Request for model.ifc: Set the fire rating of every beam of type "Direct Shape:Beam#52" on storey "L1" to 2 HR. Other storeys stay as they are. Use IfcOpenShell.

First a look at what the model holds.

```python
import ifcopenshell
import ifcopenshell.util.element

model = ifcopenshell.open("model.ifc")
print(model.schema)
storey = next(s for s in model.by_type("IfcBuildingStorey") if s.Name == "L1")
beams = [e for e in ifcopenshell.util.element.get_decomposition(storey) if e.is_a("IfcBeam")]
seen = {}
for e in beams:
    element_type = ifcopenshell.util.element.get_type(e)
    key = (element_type.Name if element_type != e and element_type else None, ifcopenshell.util.element.get_pset(e, "Pset_BeamCommon", "FireRating"))
    seen[key] = seen.get(key, 0) + 1
for (name, value), count in sorted(seen.items(), key=str):
    print(count, "x", name, "|", value)
```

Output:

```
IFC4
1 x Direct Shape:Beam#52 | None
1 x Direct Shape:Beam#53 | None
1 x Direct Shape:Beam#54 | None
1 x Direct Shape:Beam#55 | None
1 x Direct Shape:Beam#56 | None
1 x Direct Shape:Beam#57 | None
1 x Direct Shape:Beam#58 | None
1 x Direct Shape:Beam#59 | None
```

```python
import ifcopenshell
import ifcopenshell.api.pset
import ifcopenshell.util.element

model = ifcopenshell.open("model.ifc")

storey = next(s for s in model.by_type("IfcBuildingStorey") if s.Name == "L1")
beams = [e for e in ifcopenshell.util.element.get_decomposition(storey) if e.is_a("IfcBeam")]

count = 0
for e in beams:
    element_type = ifcopenshell.util.element.get_type(e)
    if element_type in (None, e) or element_type.Name != "Direct Shape:Beam#52":
        continue
    # add_pset returns the element's existing set when there is one.
    pset = ifcopenshell.api.pset.add_pset(model, product=e, name="Pset_BeamCommon")
    ifcopenshell.api.pset.edit_pset(model, pset=pset, properties={"FireRating": "2 HR"})
    count += 1

print(count, "beams updated")

model.write("model_edited.ifc")
```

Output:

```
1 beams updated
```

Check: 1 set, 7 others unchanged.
